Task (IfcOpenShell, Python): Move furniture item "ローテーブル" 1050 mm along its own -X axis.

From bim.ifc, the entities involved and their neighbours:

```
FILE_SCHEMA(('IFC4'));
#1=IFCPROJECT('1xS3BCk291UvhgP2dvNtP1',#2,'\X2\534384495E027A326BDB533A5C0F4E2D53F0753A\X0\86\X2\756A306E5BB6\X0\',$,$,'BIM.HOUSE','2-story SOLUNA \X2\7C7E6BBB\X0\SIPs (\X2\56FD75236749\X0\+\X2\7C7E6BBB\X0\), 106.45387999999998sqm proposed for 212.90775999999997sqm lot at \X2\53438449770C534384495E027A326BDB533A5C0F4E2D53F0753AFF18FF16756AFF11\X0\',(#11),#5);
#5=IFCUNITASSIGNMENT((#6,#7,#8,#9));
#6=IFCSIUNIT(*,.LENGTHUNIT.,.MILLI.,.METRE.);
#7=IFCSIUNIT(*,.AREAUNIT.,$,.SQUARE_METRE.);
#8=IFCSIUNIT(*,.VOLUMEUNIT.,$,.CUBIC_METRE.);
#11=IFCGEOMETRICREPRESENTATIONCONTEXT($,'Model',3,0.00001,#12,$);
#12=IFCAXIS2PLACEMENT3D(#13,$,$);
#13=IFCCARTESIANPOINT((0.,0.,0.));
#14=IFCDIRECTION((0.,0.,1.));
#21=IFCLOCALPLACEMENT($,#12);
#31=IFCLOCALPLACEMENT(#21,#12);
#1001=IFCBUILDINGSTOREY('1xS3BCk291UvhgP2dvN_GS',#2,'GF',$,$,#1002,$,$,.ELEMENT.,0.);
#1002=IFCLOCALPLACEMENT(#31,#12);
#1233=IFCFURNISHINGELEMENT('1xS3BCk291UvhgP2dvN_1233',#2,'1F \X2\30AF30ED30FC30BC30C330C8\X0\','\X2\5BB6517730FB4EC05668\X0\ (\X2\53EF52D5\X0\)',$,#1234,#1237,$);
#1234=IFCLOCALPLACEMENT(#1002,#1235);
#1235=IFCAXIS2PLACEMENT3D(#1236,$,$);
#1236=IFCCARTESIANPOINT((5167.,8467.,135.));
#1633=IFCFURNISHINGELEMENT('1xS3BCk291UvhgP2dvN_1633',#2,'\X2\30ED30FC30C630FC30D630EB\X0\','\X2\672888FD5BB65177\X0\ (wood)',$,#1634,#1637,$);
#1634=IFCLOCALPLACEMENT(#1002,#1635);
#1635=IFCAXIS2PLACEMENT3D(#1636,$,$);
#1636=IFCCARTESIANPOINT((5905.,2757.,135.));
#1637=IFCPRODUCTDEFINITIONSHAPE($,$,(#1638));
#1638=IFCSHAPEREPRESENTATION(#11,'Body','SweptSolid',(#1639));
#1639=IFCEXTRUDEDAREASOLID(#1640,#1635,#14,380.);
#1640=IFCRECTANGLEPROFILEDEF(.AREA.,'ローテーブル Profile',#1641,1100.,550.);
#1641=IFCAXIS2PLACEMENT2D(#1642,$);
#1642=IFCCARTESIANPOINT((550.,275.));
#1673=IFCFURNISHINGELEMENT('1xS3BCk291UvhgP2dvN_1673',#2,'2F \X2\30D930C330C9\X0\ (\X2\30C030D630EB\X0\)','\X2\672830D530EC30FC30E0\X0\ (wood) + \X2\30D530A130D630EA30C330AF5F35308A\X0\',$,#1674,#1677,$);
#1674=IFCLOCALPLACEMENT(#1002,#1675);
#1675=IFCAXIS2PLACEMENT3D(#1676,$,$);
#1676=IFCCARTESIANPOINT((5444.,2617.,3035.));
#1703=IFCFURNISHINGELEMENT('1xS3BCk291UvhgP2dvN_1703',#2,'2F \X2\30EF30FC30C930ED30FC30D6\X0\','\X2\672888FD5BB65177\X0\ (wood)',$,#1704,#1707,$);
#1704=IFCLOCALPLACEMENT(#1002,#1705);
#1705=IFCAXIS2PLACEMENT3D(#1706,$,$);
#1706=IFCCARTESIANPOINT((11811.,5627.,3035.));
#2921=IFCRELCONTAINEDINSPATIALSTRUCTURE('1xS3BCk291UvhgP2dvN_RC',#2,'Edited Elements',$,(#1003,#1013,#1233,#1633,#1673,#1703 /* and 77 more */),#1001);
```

```python
import ifcopenshell
import ifcopenshell.api.geometry
import ifcopenshell.util.placement

model = ifcopenshell.open("bim.ifc")

item = model.by_guid("1xS3BCk291UvhgP2dvN_1633")
matrix = ifcopenshell.util.placement.get_local_placement(item.ObjectPlacement)
matrix[:3, 3] -= matrix[:3, 0] * 1050.0
ifcopenshell.api.geometry.edit_object_placement(model, product=item, matrix=matrix, is_si=False)

print(ifcopenshell.util.placement.get_local_placement(item.ObjectPlacement).round(3) + 0.0)

model.write("bim_rev.ifc")
```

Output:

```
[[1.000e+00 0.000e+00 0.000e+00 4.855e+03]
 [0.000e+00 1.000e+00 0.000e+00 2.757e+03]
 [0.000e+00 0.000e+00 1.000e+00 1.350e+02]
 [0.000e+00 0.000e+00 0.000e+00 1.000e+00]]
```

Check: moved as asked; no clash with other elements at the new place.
